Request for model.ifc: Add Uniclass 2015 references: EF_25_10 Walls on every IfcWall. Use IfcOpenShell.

First a look at what the model holds.

```python
import ifcopenshell

model = ifcopenshell.open("model.ifc")
print(model.schema)
print("classifications:", [c.Name for c in model.by_type("IfcClassification")])
for ifc_class in ("IfcDoor", "IfcRoof", "IfcStair", "IfcWall", "IfcWindow"):
    print(ifc_class, len(model.by_type(ifc_class)))
```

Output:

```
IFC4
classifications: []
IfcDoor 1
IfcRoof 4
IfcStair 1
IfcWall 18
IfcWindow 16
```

```python
import ifcopenshell
import ifcopenshell.api.classification

model = ifcopenshell.open("model.ifc")

system = ifcopenshell.api.classification.add_classification(model, classification="Uniclass 2015")

codes = {
    "IfcWall": ("EF_25_10", "Walls"),
}
for ifc_class, (code, name) in codes.items():
    products = model.by_type(ifc_class)
    ifcopenshell.api.classification.add_reference(
        model, products=products, classification=system, identification=code, name=name
    )
    print(code, len(products))

model.write("model_v2.ifc")
```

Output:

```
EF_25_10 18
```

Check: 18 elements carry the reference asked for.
